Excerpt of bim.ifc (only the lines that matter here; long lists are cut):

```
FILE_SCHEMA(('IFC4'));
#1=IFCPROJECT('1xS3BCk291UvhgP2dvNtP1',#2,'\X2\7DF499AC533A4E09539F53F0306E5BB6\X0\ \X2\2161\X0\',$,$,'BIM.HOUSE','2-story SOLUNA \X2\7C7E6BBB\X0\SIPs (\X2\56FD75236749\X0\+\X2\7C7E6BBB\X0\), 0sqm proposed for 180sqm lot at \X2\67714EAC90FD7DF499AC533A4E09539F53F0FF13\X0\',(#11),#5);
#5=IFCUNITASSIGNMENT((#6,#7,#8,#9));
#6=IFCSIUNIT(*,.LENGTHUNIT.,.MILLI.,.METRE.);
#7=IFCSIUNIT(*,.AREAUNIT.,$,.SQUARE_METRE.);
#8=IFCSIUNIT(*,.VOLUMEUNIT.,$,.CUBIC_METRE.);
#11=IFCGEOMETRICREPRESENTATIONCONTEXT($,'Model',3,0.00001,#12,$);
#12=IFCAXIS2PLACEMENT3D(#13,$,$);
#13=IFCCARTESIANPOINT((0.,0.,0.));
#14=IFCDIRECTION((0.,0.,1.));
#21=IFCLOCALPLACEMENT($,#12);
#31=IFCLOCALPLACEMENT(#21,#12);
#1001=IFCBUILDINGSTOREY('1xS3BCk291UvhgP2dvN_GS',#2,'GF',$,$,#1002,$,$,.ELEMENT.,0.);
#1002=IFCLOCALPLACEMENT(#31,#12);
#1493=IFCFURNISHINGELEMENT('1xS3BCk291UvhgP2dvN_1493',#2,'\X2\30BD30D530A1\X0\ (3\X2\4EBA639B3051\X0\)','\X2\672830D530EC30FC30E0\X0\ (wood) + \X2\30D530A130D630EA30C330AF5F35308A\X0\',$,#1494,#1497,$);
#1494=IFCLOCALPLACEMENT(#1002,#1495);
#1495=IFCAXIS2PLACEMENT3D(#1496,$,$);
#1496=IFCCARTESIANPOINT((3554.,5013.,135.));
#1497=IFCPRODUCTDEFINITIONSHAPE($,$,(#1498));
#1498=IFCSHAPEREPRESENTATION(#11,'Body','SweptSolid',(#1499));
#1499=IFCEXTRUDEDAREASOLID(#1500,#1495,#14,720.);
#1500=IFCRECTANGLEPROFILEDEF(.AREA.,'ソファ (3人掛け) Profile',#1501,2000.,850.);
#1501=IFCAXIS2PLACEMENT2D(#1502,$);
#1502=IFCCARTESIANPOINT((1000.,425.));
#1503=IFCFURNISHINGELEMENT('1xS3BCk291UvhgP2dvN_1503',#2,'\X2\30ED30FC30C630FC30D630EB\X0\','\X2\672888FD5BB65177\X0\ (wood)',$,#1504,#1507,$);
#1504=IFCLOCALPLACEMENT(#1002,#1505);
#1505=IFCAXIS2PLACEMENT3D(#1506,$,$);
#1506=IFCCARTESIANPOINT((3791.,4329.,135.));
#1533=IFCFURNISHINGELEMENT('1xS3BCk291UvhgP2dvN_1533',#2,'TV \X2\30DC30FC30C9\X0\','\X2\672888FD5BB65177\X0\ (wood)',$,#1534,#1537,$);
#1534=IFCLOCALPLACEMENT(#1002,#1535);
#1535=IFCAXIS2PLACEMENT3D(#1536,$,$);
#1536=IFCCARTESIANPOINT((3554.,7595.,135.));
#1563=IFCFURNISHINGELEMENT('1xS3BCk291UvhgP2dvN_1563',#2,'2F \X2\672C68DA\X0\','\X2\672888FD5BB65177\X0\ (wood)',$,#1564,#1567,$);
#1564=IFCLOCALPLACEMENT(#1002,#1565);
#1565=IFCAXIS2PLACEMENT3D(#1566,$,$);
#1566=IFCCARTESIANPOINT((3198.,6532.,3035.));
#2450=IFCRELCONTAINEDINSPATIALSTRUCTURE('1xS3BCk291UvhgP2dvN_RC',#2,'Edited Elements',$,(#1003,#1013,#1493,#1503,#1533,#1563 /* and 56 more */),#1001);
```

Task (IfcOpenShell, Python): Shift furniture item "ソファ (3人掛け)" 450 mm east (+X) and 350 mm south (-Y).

```python
import ifcopenshell
import ifcopenshell.api.geometry
import ifcopenshell.util.placement

model = ifcopenshell.open("bim.ifc")

item = model.by_guid("1xS3BCk291UvhgP2dvN_1493")
matrix = ifcopenshell.util.placement.get_local_placement(item.ObjectPlacement)
matrix[0, 3] += 450.0
matrix[1, 3] -= 350.0
ifcopenshell.api.geometry.edit_object_placement(model, product=item, matrix=matrix, is_si=False)

print(ifcopenshell.util.placement.get_local_placement(item.ObjectPlacement).round(3) + 0.0)

model.write("bim_rev.ifc")
```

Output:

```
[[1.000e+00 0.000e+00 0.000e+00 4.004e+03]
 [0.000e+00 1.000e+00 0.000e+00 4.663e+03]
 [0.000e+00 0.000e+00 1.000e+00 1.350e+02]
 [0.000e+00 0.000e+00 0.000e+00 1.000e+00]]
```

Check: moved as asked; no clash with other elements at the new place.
